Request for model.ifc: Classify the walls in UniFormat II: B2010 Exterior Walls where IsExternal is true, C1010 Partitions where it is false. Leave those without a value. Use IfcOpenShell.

First a look at what the model holds.

```python
import ifcopenshell
import ifcopenshell.util.element

model = ifcopenshell.open("model.ifc")
print(model.schema)
print("classifications:", [c.Name for c in model.by_type("IfcClassification")])
values = [ifcopenshell.util.element.get_pset(e, "Pset_WallCommon", "IsExternal") for e in model.by_type("IfcWall")]
for value in (True, False, None):
    print("IsExternal", value, values.count(value))
```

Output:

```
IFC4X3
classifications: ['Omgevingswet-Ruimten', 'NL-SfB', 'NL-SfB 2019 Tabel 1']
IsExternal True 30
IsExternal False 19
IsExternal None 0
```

```python
import ifcopenshell
import ifcopenshell.api.classification
import ifcopenshell.util.element

model = ifcopenshell.open("model.ifc")

system = ifcopenshell.api.classification.add_classification(model, classification="UniFormat II")

walls = model.by_type("IfcWall")
external = {e: ifcopenshell.util.element.get_pset(e, "Pset_WallCommon", "IsExternal") for e in walls}
for flag, code, name in ((True, "B2010", "Exterior Walls"), (False, "C1010", "Partitions")):
    products = [e for e in walls if external[e] is flag]
    ifcopenshell.api.classification.add_reference(
        model, products=products, classification=system, identification=code, name=name
    )
    print(code, len(products))

model.write("model_v2.ifc")
```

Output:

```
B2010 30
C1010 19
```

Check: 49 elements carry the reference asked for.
